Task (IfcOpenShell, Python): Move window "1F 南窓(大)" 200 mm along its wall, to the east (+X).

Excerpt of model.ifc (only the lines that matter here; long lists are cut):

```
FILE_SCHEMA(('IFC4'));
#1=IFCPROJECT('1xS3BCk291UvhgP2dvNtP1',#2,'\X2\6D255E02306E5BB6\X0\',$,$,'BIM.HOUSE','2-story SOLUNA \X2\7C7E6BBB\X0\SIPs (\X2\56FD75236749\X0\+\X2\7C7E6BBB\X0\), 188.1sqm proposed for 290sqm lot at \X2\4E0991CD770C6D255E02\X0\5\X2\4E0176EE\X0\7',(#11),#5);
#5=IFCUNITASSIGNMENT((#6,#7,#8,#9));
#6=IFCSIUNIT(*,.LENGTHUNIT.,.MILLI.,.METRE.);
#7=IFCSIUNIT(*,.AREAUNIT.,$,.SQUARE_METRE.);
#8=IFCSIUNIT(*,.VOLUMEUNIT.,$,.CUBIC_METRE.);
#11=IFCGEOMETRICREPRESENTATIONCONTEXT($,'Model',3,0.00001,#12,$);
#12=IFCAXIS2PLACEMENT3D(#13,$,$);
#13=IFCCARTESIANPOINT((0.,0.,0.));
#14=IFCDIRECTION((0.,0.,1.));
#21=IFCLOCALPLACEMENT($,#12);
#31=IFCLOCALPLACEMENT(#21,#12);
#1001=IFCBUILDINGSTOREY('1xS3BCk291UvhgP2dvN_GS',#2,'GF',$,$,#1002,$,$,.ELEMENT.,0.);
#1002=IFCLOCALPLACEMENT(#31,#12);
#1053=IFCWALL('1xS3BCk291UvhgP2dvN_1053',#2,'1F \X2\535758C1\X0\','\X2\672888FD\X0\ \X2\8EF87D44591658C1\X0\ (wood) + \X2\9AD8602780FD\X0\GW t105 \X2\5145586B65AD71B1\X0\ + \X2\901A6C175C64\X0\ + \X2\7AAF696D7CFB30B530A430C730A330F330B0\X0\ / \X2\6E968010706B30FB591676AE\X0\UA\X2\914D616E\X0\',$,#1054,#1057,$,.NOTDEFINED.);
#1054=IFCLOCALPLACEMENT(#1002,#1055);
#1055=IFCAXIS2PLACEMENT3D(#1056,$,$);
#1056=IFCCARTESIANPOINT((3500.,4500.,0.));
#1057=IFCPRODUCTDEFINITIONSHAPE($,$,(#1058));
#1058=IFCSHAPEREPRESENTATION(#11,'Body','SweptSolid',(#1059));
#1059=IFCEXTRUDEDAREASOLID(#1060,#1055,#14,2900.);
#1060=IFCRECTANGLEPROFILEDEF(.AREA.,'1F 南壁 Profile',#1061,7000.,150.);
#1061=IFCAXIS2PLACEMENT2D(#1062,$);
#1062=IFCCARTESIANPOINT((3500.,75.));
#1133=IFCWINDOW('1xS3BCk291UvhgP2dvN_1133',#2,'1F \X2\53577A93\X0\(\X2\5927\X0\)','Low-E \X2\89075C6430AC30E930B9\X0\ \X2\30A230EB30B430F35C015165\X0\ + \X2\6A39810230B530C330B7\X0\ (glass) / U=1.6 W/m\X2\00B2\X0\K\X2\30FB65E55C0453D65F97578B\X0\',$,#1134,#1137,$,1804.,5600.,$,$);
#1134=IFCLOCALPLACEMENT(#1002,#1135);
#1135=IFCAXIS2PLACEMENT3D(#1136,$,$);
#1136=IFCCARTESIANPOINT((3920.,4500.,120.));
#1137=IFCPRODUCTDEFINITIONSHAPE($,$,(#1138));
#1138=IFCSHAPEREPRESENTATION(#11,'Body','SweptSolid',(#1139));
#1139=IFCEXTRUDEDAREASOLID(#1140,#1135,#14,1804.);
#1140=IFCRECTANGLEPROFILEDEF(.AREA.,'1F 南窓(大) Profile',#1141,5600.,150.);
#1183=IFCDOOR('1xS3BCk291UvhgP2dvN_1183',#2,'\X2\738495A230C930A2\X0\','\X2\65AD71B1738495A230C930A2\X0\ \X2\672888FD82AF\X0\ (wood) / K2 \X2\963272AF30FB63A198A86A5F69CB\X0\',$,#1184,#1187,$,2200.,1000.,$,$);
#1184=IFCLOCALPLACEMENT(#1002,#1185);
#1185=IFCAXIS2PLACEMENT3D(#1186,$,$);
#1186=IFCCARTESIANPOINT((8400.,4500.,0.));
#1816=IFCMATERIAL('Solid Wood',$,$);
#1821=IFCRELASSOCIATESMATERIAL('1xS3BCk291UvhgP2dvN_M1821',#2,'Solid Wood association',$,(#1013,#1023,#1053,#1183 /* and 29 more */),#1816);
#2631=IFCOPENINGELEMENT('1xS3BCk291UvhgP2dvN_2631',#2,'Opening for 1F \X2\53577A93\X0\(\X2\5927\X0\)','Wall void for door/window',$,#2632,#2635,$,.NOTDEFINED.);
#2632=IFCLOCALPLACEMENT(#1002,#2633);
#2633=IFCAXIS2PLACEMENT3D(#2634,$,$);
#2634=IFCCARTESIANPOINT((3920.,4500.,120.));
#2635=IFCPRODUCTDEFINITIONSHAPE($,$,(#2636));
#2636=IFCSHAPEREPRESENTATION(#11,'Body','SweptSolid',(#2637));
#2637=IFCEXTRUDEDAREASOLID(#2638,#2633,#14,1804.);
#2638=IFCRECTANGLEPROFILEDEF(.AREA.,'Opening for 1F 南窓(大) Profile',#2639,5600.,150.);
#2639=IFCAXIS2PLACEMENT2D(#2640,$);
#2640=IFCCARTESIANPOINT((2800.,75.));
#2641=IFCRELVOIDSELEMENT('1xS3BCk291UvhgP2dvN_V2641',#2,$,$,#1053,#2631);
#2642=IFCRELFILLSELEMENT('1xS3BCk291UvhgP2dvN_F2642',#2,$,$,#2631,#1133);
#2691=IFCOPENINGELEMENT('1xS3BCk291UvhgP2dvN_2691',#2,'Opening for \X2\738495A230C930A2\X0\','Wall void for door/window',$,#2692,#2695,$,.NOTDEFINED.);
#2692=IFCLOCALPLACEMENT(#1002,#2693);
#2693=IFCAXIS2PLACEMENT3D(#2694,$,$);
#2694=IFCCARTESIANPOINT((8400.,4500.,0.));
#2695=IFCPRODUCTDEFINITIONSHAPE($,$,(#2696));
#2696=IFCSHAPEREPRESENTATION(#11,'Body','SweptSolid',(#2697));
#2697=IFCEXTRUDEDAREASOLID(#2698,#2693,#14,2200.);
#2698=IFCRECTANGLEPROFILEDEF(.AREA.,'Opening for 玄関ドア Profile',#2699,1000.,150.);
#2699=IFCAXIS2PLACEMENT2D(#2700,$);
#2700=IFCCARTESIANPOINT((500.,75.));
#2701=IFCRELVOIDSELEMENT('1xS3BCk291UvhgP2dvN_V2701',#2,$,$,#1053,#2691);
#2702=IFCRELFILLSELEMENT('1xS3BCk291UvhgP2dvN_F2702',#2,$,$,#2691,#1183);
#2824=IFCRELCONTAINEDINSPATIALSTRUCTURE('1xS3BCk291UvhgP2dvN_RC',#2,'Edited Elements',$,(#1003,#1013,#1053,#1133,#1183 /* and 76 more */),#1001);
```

```python
import ifcopenshell
import ifcopenshell.api.geometry
import ifcopenshell.util.placement

model = ifcopenshell.open("model.ifc")

window = model.by_guid("1xS3BCk291UvhgP2dvN_1133")
opening = window.FillsVoids[0].RelatingOpeningElement
wall = opening.VoidsElements[0].RelatingBuildingElement

wall_matrix = ifcopenshell.util.placement.get_local_placement(wall.ObjectPlacement)
shift = wall_matrix[:3, 0] * 200.0
before = ifcopenshell.util.placement.get_local_placement(window.ObjectPlacement)[:3, 3].copy()

# The window is not placed relative to its opening, so move both.
for product in (opening, window):
    matrix = ifcopenshell.util.placement.get_local_placement(product.ObjectPlacement)
    matrix[:3, 3] += shift
    ifcopenshell.api.geometry.edit_object_placement(model, product=product, matrix=matrix, is_si=False)

after = ifcopenshell.util.placement.get_local_placement(window.ObjectPlacement)[:3, 3]
print("window moved by", (after - before).round(3) + 0.0)

model.write("model_rev.ifc")
```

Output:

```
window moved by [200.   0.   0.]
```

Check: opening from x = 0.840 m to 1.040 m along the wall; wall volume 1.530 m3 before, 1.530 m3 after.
